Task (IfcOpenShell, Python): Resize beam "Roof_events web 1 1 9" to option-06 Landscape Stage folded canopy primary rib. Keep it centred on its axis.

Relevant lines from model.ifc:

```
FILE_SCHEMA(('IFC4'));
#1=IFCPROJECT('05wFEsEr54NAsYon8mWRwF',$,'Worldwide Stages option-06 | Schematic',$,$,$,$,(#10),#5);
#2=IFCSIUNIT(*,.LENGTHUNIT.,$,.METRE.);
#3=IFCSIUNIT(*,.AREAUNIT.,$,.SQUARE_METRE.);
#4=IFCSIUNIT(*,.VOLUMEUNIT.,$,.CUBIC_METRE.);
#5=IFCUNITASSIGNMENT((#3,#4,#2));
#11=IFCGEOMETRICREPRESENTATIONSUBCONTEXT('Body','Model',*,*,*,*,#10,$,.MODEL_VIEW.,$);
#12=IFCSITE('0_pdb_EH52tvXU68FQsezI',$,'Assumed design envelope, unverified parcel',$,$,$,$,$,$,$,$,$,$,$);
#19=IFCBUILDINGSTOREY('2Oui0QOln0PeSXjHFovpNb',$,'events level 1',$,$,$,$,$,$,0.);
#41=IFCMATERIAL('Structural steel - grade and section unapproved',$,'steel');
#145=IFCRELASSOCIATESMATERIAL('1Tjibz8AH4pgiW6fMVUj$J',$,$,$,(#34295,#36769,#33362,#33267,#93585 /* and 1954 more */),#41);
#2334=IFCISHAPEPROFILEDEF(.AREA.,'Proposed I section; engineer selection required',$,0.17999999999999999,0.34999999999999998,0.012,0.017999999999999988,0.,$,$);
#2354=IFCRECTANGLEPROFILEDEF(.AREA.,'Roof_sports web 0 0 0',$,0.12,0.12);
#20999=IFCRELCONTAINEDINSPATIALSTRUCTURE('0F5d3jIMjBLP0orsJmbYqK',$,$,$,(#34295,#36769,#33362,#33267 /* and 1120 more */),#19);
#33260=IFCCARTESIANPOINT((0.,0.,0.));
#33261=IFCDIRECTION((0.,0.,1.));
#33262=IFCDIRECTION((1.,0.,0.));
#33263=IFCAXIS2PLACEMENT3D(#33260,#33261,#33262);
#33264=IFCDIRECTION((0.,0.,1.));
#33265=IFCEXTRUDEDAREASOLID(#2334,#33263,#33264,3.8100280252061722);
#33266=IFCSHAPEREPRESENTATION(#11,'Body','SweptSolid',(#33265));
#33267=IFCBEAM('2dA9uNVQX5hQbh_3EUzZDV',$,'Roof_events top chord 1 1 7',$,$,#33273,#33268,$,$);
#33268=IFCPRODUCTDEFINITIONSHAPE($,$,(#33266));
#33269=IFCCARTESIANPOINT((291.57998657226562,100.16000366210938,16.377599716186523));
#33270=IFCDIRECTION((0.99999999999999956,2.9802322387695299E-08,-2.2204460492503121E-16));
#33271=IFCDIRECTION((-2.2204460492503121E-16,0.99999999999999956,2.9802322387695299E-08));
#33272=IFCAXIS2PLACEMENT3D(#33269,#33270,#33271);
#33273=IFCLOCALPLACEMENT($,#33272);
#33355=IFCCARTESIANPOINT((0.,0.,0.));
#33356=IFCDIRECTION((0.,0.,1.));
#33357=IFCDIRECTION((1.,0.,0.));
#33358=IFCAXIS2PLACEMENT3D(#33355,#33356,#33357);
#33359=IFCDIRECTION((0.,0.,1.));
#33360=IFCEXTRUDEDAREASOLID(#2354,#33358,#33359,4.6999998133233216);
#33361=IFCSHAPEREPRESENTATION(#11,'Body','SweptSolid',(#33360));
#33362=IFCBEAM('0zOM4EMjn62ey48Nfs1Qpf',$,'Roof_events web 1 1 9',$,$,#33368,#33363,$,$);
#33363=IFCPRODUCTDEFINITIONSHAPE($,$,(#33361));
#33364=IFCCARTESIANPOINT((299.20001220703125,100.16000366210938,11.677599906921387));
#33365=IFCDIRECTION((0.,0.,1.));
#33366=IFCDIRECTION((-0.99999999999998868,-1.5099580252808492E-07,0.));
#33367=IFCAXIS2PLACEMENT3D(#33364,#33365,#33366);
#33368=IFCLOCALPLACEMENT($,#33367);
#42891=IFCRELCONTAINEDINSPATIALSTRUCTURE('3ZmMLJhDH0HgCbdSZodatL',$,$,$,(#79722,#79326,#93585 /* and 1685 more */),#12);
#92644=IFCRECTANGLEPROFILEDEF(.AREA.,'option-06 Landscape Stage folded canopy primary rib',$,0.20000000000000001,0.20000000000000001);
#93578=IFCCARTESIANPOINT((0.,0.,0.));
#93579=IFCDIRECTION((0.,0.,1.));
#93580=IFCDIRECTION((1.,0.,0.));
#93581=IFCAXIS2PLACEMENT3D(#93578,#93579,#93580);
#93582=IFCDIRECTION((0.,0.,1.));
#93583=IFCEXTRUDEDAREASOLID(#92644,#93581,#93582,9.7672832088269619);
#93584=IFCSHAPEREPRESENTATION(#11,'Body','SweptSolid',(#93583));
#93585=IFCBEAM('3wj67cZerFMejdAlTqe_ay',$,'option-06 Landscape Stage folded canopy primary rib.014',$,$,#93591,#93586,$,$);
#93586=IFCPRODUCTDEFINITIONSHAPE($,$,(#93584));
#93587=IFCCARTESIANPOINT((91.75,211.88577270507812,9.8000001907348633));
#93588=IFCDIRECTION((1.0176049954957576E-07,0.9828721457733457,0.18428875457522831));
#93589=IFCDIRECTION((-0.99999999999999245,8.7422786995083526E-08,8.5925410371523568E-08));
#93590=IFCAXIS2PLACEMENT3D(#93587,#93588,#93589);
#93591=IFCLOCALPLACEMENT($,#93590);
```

```python
import ifcopenshell
import ifcopenshell.util.element
import ifcopenshell.util.representation

model = ifcopenshell.open("model.ifc")

member = model.by_id(33362)
source = next(p for p in model.by_type("IfcRectangleProfileDef") if p.ProfileName == "option-06 Landscape Stage folded canopy primary rib")

body = ifcopenshell.util.representation.get_representation(member, "Model", "Body")
solid = body.Items[0]
old_profile = solid.SweptArea

# Copy the section's sizes but keep this member's own profile position.
profile = ifcopenshell.util.element.copy(model, source)
profile.Position = old_profile.Position
solid.SweptArea = profile
if not model.get_total_inverses(old_profile):
    ifcopenshell.util.element.remove_deep2(model, old_profile)

print(solid.SweptArea)

model.write("model_updated.ifc")
```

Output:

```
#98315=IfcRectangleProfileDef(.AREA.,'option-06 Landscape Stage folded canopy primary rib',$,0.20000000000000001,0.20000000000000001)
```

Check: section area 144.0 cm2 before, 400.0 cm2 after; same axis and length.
